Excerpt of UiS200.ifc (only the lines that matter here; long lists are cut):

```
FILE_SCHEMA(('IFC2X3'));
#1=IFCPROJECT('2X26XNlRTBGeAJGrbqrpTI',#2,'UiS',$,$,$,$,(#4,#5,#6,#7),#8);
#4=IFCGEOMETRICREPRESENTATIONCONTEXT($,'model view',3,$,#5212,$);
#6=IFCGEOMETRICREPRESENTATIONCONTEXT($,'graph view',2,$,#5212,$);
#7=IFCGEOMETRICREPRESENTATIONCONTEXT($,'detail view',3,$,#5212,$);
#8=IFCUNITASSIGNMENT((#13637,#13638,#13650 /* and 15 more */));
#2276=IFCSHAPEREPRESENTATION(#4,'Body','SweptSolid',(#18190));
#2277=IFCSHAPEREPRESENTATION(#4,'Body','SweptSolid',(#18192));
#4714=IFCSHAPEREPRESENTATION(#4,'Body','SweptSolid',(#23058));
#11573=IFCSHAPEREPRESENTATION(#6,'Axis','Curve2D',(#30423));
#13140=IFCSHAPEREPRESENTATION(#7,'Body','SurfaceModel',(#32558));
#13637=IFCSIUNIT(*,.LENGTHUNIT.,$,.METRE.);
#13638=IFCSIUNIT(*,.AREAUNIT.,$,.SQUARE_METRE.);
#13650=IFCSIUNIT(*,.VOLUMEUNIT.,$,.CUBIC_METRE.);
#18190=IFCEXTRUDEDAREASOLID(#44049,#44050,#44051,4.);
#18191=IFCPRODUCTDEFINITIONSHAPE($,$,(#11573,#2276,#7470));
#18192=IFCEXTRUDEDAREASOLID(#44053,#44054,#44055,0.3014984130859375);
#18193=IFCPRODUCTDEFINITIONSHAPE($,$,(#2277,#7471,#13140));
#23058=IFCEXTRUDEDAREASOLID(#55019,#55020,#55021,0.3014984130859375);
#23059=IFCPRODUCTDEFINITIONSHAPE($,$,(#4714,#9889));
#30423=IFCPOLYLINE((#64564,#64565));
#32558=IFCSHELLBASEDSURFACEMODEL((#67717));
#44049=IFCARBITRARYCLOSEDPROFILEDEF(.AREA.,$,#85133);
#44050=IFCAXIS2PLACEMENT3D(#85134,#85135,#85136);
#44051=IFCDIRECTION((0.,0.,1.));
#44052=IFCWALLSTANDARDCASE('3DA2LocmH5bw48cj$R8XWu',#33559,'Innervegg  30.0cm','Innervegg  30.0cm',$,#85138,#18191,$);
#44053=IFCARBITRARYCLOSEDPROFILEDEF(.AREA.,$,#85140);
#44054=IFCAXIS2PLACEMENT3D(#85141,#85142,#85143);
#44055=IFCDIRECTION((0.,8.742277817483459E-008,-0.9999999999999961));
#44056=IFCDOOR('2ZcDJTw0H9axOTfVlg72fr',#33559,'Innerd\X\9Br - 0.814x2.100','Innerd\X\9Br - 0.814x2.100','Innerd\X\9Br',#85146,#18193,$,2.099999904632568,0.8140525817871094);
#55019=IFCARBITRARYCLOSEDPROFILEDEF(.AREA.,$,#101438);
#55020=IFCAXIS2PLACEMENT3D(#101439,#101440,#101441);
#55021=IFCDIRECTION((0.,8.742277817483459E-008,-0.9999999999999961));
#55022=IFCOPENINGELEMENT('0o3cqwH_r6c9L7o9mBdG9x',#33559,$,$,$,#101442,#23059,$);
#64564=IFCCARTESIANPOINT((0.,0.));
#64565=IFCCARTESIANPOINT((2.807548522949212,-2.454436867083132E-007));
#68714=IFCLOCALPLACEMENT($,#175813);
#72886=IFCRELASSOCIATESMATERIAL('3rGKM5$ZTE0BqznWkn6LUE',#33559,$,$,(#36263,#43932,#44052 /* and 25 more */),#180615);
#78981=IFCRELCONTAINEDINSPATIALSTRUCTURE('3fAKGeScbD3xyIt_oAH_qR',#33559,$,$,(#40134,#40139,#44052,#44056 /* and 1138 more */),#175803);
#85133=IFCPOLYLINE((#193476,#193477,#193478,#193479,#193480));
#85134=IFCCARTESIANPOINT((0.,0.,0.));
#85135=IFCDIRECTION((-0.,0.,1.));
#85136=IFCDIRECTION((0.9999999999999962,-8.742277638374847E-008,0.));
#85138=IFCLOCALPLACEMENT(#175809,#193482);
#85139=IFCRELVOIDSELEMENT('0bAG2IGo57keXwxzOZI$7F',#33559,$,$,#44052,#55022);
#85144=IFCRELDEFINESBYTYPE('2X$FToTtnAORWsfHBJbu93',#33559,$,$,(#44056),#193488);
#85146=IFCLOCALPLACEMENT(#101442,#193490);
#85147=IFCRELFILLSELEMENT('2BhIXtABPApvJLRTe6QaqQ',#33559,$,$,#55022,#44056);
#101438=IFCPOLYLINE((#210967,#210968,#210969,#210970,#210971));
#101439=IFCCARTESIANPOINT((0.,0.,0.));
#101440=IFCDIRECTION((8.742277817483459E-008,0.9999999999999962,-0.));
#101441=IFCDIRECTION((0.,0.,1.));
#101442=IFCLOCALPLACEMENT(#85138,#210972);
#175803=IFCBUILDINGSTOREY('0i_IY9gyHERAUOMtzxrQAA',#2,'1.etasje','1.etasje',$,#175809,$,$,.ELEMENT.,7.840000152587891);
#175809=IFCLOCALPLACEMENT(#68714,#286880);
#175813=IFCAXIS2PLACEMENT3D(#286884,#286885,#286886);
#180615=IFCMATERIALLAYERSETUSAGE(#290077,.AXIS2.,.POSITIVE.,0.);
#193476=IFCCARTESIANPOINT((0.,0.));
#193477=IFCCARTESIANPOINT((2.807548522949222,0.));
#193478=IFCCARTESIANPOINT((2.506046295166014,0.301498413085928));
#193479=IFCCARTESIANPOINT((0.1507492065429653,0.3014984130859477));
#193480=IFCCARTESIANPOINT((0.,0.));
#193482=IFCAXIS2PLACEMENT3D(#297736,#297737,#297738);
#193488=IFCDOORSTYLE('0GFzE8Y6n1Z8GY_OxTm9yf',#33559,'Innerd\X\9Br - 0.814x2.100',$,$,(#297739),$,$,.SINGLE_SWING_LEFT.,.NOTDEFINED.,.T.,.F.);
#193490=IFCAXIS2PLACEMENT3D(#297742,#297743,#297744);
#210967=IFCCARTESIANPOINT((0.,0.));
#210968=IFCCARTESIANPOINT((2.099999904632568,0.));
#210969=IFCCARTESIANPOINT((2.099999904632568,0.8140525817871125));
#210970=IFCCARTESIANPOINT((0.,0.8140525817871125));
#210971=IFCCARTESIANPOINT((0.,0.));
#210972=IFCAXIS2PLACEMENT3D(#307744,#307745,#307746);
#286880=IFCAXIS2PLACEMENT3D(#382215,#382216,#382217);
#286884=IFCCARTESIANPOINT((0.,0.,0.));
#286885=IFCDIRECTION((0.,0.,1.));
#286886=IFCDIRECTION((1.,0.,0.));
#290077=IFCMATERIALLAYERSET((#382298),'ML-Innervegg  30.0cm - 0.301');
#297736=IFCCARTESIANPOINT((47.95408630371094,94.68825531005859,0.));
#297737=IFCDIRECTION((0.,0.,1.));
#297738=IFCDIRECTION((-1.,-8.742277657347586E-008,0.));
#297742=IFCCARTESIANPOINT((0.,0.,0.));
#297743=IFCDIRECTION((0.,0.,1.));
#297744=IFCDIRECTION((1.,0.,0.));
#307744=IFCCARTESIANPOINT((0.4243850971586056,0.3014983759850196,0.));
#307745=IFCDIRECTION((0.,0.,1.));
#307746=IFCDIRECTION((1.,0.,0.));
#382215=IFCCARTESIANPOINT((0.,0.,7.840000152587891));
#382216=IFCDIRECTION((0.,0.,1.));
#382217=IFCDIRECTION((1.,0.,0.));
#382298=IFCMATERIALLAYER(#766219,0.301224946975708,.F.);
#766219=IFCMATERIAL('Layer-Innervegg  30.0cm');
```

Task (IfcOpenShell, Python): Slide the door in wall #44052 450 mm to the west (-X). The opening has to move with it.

```python
import ifcopenshell
import ifcopenshell.api.geometry
import ifcopenshell.util.placement
import ifcopenshell.util.unit

model = ifcopenshell.open("UiS200.ifc")
unit_scale = ifcopenshell.util.unit.calculate_unit_scale(model)

door = model.by_guid("2ZcDJTw0H9axOTfVlg72fr")
opening = door.FillsVoids[0].RelatingOpeningElement
wall = opening.VoidsElements[0].RelatingBuildingElement

wall_matrix = ifcopenshell.util.placement.get_local_placement(wall.ObjectPlacement)
shift = wall_matrix[:3, 0] * 0.45 / unit_scale
before = ifcopenshell.util.placement.get_local_placement(door.ObjectPlacement)[:3, 3].copy()

# The door is placed relative to its opening, so it follows when the opening moves.
matrix = ifcopenshell.util.placement.get_local_placement(opening.ObjectPlacement)
matrix[:3, 3] += shift
ifcopenshell.api.geometry.edit_object_placement(
    model, product=opening, matrix=matrix, is_si=False, should_transform_children=True
)

after = ifcopenshell.util.placement.get_local_placement(door.ObjectPlacement)[:3, 3]
print("door moved by", (after - before).round(3) + 0.0)

model.write("UiS200_edited.ifc")
```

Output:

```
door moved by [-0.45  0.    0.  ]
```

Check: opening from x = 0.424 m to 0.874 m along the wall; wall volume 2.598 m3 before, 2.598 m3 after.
